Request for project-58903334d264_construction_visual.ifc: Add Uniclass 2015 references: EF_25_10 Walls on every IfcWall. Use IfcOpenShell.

First a look at what the model holds.

```python
import ifcopenshell

model = ifcopenshell.open("project-58903334d264_construction_visual.ifc")
print(model.schema)
print("classifications:", [c.Name for c in model.by_type("IfcClassification")])
for ifc_class in ("IfcDoor", "IfcRoof", "IfcStair", "IfcWall", "IfcWindow"):
    print(ifc_class, len(model.by_type(ifc_class)))
```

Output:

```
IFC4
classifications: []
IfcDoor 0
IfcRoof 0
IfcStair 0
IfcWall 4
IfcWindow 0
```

```python
import ifcopenshell
import ifcopenshell.api.classification

model = ifcopenshell.open("project-58903334d264_construction_visual.ifc")

system = ifcopenshell.api.classification.add_classification(model, classification="Uniclass 2015")

codes = {
    "IfcWall": ("EF_25_10", "Walls"),
}
for ifc_class, (code, name) in codes.items():
    products = model.by_type(ifc_class)
    ifcopenshell.api.classification.add_reference(
        model, products=products, classification=system, identification=code, name=name
    )
    print(code, len(products))

model.write("project-58903334d264_construction_visual_edited.ifc")
```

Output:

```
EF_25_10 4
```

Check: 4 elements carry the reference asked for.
